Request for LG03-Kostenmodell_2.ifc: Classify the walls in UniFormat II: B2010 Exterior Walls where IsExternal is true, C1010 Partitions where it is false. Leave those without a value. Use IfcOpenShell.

First a look at what the model holds.

```python
import ifcopenshell
import ifcopenshell.util.element

model = ifcopenshell.open("LG03-Kostenmodell_2.ifc")
print(model.schema)
print("classifications:", [c.Name for c in model.by_type("IfcClassification")])
values = [ifcopenshell.util.element.get_pset(e, "Pset_WallCommon", "IsExternal") for e in model.by_type("IfcWall")]
for value in (True, False, None):
    print("IsExternal", value, values.count(value))
```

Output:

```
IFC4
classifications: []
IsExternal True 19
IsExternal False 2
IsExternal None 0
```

```python
import ifcopenshell
import ifcopenshell.api.classification
import ifcopenshell.util.element

model = ifcopenshell.open("LG03-Kostenmodell_2.ifc")

system = ifcopenshell.api.classification.add_classification(model, classification="UniFormat II")

walls = model.by_type("IfcWall")
external = {e: ifcopenshell.util.element.get_pset(e, "Pset_WallCommon", "IsExternal") for e in walls}
for flag, code, name in ((True, "B2010", "Exterior Walls"), (False, "C1010", "Partitions")):
    products = [e for e in walls if external[e] is flag]
    ifcopenshell.api.classification.add_reference(
        model, products=products, classification=system, identification=code, name=name
    )
    print(code, len(products))

model.write("LG03-Kostenmodell_2_edited.ifc")
```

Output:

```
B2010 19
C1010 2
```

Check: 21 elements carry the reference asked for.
